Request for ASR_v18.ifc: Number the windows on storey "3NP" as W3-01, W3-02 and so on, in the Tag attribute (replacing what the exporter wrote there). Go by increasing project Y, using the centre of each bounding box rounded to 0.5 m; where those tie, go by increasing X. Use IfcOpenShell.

First a look at what the model holds.

```python
import ifcopenshell
import ifcopenshell.util.element
import ifcopenshell.util.placement

model = ifcopenshell.open("ASR_v18.ifc")
print(model.schema)
storey = next(s for s in model.by_type("IfcBuildingStorey") if s.Name == "3NP")
windows = [e for e in ifcopenshell.util.element.get_decomposition(storey) if e.is_a("IfcWindow")]
for e in sorted(windows, key=lambda e: e.id()):
    origin = ifcopenshell.util.placement.get_local_placement(e.ObjectPlacement)[:3, 3]
    print(e.id(), e.Tag, e.Name, origin.round(2) + 0.0, sep=" | ")
```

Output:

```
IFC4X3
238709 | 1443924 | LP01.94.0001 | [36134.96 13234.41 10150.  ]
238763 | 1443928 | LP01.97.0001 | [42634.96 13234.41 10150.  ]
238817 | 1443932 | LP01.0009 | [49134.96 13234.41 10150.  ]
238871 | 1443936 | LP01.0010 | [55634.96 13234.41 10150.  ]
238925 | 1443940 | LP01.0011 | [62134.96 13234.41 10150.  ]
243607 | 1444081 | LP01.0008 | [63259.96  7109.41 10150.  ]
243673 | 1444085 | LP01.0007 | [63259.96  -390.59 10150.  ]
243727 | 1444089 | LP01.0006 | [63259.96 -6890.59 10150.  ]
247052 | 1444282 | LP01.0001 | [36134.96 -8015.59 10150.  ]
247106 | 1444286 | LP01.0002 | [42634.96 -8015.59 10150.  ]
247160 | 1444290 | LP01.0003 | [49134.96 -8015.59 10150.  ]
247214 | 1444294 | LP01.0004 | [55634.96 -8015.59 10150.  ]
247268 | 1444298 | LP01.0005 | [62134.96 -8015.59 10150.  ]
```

```python
import ifcopenshell
import ifcopenshell.geom
import ifcopenshell.util.element
import ifcopenshell.util.shape

model = ifcopenshell.open("ASR_v18.ifc")
settings = ifcopenshell.geom.settings()
settings.set("use-world-coords", True)


def centre(element):
    shape = ifcopenshell.geom.create_shape(settings, element)
    return ifcopenshell.util.shape.get_bbox_centroid(shape.geometry)


storey = next(s for s in model.by_type("IfcBuildingStorey") if s.Name == "3NP")
windows = [e for e in ifcopenshell.util.element.get_decomposition(storey) if e.is_a("IfcWindow")]

# Insertion points can sit at a corner or the storey origin, so sort by the geometry (in metres).
centres = {e: centre(e) for e in windows}
windows.sort(key=lambda e: (round(centres[e][1] / 0.5), centres[e][0]))

for i, e in enumerate(windows, start=1):
    number = f"W3-{i:02d}"
    e.Tag = number
    print(e.id(), number)

model.write("ASR_v18_updated.ifc")
```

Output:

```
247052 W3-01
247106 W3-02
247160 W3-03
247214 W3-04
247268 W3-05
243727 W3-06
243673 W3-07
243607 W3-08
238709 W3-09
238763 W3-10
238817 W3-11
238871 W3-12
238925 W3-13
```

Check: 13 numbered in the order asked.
